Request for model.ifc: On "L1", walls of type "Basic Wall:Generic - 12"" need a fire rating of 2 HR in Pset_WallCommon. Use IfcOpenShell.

First a look at what the model holds.

```python
import ifcopenshell
import ifcopenshell.util.element

model = ifcopenshell.open("model.ifc")
print(model.schema)
storey = next(s for s in model.by_type("IfcBuildingStorey") if s.Name == "L1")
walls = [e for e in ifcopenshell.util.element.get_decomposition(storey) if e.is_a("IfcWall")]
seen = {}
for e in walls:
    element_type = ifcopenshell.util.element.get_type(e)
    key = (element_type.Name if element_type != e and element_type else None, ifcopenshell.util.element.get_pset(e, "Pset_WallCommon", "FireRating"))
    seen[key] = seen.get(key, 0) + 1
for (name, value), count in sorted(seen.items(), key=str):
    print(count, "x", name, "|", value)
```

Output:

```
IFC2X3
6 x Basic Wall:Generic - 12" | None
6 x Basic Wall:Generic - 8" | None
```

```python
import ifcopenshell
import ifcopenshell.api.pset
import ifcopenshell.util.element

model = ifcopenshell.open("model.ifc")

storey = next(s for s in model.by_type("IfcBuildingStorey") if s.Name == "L1")
walls = [e for e in ifcopenshell.util.element.get_decomposition(storey) if e.is_a("IfcWall")]

count = 0
for e in walls:
    element_type = ifcopenshell.util.element.get_type(e)
    if element_type in (None, e) or element_type.Name != 'Basic Wall:Generic - 12"':
        continue
    # add_pset returns the element's existing set when there is one.
    pset = ifcopenshell.api.pset.add_pset(model, product=e, name="Pset_WallCommon")
    ifcopenshell.api.pset.edit_pset(model, pset=pset, properties={"FireRating": "2 HR"})
    count += 1

print(count, "walls updated")

model.write("model_v2.ifc")
```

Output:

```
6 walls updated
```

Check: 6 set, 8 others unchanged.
